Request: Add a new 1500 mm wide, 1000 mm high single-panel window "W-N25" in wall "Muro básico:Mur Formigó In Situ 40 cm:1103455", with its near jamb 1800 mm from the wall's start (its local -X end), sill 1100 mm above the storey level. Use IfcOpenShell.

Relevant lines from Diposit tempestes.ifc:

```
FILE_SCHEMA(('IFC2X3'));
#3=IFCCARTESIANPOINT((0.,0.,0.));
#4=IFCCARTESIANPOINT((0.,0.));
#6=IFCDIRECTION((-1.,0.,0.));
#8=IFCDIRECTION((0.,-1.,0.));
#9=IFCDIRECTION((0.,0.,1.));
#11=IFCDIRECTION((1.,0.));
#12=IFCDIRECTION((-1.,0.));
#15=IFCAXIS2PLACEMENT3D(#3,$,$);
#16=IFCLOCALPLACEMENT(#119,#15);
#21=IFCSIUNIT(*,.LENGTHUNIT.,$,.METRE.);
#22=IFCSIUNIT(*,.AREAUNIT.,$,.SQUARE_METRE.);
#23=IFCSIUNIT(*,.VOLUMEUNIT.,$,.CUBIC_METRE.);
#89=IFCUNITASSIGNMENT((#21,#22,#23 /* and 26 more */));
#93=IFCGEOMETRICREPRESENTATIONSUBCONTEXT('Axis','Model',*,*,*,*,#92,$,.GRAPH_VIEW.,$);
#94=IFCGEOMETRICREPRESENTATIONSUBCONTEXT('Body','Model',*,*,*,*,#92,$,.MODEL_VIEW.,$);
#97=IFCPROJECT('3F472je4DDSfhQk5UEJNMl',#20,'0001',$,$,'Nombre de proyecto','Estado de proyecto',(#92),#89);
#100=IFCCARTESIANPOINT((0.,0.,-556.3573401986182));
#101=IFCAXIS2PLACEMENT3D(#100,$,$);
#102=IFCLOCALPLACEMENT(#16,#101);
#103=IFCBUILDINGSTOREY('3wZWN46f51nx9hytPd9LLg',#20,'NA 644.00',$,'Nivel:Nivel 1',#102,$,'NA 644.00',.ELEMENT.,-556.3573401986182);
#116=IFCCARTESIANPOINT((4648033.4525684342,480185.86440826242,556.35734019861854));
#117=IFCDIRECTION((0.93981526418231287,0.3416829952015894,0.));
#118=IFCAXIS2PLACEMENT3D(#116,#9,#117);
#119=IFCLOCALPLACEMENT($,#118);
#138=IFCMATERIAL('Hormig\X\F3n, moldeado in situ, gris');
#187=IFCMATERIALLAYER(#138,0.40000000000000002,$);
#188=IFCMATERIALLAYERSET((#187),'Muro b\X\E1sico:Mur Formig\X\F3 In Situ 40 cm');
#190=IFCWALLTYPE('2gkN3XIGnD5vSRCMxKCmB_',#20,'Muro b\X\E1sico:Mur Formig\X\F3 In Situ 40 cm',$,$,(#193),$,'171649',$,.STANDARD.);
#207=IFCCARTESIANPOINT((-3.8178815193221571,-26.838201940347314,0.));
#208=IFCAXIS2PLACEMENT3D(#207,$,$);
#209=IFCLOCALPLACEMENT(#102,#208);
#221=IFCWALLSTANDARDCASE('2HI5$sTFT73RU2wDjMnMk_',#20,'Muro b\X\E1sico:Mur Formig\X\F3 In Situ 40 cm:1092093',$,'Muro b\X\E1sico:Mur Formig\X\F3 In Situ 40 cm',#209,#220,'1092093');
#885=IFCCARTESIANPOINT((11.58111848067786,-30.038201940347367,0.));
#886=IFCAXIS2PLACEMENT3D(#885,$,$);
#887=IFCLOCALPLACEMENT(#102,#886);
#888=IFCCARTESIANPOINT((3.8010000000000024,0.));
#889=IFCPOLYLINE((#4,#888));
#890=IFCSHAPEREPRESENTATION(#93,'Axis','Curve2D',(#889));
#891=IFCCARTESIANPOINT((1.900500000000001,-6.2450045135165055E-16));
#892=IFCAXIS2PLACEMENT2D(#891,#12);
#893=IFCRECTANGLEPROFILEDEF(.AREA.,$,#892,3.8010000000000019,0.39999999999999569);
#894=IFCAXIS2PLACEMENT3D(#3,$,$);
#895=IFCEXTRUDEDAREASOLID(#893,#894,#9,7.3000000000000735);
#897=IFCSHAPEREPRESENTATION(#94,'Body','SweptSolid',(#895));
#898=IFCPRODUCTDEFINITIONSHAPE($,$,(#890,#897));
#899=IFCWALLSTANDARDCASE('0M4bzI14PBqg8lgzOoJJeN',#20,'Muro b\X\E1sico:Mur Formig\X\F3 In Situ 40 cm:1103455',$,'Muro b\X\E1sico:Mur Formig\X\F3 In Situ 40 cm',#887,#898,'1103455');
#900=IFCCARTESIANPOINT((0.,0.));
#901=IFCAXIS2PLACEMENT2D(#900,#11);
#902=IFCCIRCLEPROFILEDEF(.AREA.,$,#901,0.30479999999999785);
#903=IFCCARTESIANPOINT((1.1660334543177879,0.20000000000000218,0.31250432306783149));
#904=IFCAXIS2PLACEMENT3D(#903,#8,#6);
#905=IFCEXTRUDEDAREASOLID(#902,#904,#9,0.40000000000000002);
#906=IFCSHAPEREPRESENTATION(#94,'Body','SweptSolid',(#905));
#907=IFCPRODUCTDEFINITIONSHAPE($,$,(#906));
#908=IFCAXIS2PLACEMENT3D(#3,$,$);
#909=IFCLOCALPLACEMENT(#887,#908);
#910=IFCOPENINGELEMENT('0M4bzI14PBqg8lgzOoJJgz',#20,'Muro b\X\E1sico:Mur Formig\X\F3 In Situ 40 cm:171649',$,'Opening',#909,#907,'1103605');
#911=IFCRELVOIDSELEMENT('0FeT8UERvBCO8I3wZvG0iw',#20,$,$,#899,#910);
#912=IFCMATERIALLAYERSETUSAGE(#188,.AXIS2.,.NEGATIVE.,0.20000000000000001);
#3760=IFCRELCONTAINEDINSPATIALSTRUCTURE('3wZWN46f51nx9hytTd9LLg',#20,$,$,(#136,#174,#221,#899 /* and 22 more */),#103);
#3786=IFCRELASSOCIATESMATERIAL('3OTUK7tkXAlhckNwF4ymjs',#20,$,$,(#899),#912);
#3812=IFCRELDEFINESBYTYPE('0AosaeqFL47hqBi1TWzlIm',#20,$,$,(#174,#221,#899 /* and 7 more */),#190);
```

```python
import numpy as np
import ifcopenshell
import ifcopenshell.api.feature
import ifcopenshell.api.geometry
import ifcopenshell.api.root
import ifcopenshell.api.spatial
import ifcopenshell.api.type
import ifcopenshell.geom
import ifcopenshell.util.element
import ifcopenshell.util.placement
import ifcopenshell.util.representation
import ifcopenshell.util.shape
import ifcopenshell.util.unit

model = ifcopenshell.open("Diposit tempestes.ifc")
unit_scale = ifcopenshell.util.unit.calculate_unit_scale(model)
settings = ifcopenshell.geom.settings()


def volume(element):
    """Net volume in cubic metres, openings subtracted."""
    shape = ifcopenshell.geom.create_shape(settings, element)
    return ifcopenshell.util.shape.get_volume(shape.geometry)


wall = model.by_id(899)
storey = ifcopenshell.util.element.get_container(wall, ifc_class="IfcBuildingStorey")
context = ifcopenshell.util.representation.get_context(model, "Model", "Body", "MODEL_VIEW")
before = volume(wall)

width, height, from_end, sill = 1.5, 1, 1.8, 1.1  # metres

# The wall runs along its own X axis, and the end named is its -X end.
wall_shape = ifcopenshell.geom.create_shape(settings, wall)
x, y, z = ifcopenshell.util.shape.get_vertices(wall_shape.geometry).T
start = x.min() + from_end
face, thickness = float(y.min()), float(y.max() - y.min())
wall_matrix = ifcopenshell.util.placement.get_local_placement(wall.ObjectPlacement)
level = ifcopenshell.util.placement.get_local_placement(storey.ObjectPlacement)[2, 3]


def in_wall(x, y):
    """Placement at x, y metres in the wall's axes, at sill height."""
    matrix = wall_matrix.copy()
    matrix[:, 3] = wall_matrix @ np.array([x / unit_scale, y / unit_scale, 0.0, 1.0])
    matrix[2, 3] = level + sill / unit_scale
    return matrix


# Opening: a box that overshoots both wall faces by 50 mm.
opening = ifcopenshell.api.root.create_entity(model, ifc_class="IfcOpeningElement")
box = ifcopenshell.api.geometry.add_wall_representation(
    model, context=context, length=width, height=height, thickness=thickness + 0.1
)
ifcopenshell.api.geometry.assign_representation(model, product=opening, representation=box)
ifcopenshell.api.geometry.edit_object_placement(model, product=opening, matrix=in_wall(start, face - 0.05), is_si=False)
ifcopenshell.api.feature.add_feature(model, feature=opening, element=wall)

window = ifcopenshell.api.root.create_entity(model, ifc_class="IfcWindow", name="W-N25")
window.OverallWidth, window.OverallHeight = width / unit_scale, height / unit_scale
body = ifcopenshell.api.geometry.add_window_representation(
    model,
    context=context,
    overall_width=window.OverallWidth,
    overall_height=window.OverallHeight,
    partition_type="SINGLE_PANEL",
)
ifcopenshell.api.geometry.assign_representation(model, product=window, representation=body)
ifcopenshell.api.spatial.assign_container(model, products=[window], relating_structure=storey)
fills = ifcopenshell.api.feature.add_filling(model, opening=opening, element=window)
fills.OwnerHistory = window.OwnerHistory  # required in IFC2X3

# IFC2X3 keeps the operation on the window style.
style = ifcopenshell.api.root.create_entity(model, ifc_class="IfcWindowStyle", name="W-N25")
style.OperationType, style.ConstructionType = "SINGLE_PANEL", "NOTDEFINED"
style.ParameterTakesPrecedence = style.Sizeable = False
ifcopenshell.api.type.assign_type(model, related_objects=[window], relating_type=style)

# Centre the window in the wall's thickness.
ifcopenshell.api.geometry.edit_object_placement(model, product=window, matrix=in_wall(start, face), is_si=False)
window_shape = ifcopenshell.geom.create_shape(settings, window)
depth = ifcopenshell.util.shape.get_vertices(window_shape.geometry)[:, 1]
offset = face + thickness / 2 - (depth.min() + depth.max()) / 2
ifcopenshell.api.geometry.edit_object_placement(model, product=window, matrix=in_wall(start, offset), is_si=False)

after = volume(wall)

print(f"wall volume {before:.3f} -> {after:.3f} m3")

model.write("Diposit tempestes_rev.ifc")
```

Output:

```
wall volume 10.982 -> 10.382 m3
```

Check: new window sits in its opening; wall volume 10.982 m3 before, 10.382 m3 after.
